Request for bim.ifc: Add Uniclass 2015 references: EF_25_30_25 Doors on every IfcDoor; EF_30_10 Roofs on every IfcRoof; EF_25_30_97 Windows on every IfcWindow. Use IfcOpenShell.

First a look at what the model holds.

```python
import ifcopenshell

model = ifcopenshell.open("bim.ifc")
print(model.schema)
print("classifications:", [c.Name for c in model.by_type("IfcClassification")])
for ifc_class in ("IfcDoor", "IfcRoof", "IfcStair", "IfcWall", "IfcWindow"):
    print(ifc_class, len(model.by_type(ifc_class)))
```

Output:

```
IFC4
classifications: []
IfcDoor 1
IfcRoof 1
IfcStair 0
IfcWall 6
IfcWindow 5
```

```python
import ifcopenshell
import ifcopenshell.api.classification

model = ifcopenshell.open("bim.ifc")

system = ifcopenshell.api.classification.add_classification(model, classification="Uniclass 2015")

codes = {
    "IfcDoor": ("EF_25_30_25", "Doors"),
    "IfcRoof": ("EF_30_10", "Roofs"),
    "IfcWindow": ("EF_25_30_97", "Windows"),
}
for ifc_class, (code, name) in codes.items():
    products = model.by_type(ifc_class)
    ifcopenshell.api.classification.add_reference(
        model, products=products, classification=system, identification=code, name=name
    )
    print(code, len(products))

model.write("bim_v2.ifc")
```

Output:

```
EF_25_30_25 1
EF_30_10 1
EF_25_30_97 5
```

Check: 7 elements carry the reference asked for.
